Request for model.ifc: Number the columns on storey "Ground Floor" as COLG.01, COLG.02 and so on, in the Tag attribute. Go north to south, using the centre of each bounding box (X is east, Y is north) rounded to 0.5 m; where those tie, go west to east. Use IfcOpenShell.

First a look at what the model holds.

```python
import ifcopenshell
import ifcopenshell.util.element
import ifcopenshell.util.placement

model = ifcopenshell.open("model.ifc")
print(model.schema)
storey = next(s for s in model.by_type("IfcBuildingStorey") if s.Name == "Ground Floor")
columns = [e for e in ifcopenshell.util.element.get_decomposition(storey) if e.is_a("IfcColumn")]
for e in sorted(columns, key=lambda e: e.id()):
    origin = ifcopenshell.util.placement.get_local_placement(e.ObjectPlacement)[:3, 3]
    print(e.id(), e.Tag, e.Name, origin.round(2) + 0.0, sep=" | ")
```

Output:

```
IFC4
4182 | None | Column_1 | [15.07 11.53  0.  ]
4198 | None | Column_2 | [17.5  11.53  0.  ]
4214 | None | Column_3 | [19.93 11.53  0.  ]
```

```python
import ifcopenshell
import ifcopenshell.geom
import ifcopenshell.util.element
import ifcopenshell.util.shape

model = ifcopenshell.open("model.ifc")
settings = ifcopenshell.geom.settings()
settings.set("use-world-coords", True)


def centre(element):
    shape = ifcopenshell.geom.create_shape(settings, element)
    return ifcopenshell.util.shape.get_bbox_centroid(shape.geometry)


storey = next(s for s in model.by_type("IfcBuildingStorey") if s.Name == "Ground Floor")
columns = [e for e in ifcopenshell.util.element.get_decomposition(storey) if e.is_a("IfcColumn")]

# Insertion points can sit at a corner or the storey origin, so sort by the geometry (in metres).
centres = {e: centre(e) for e in columns}
columns.sort(key=lambda e: (-round(centres[e][1] / 0.5), centres[e][0]))

for i, e in enumerate(columns, start=1):
    number = f"COLG.{i:02d}"
    e.Tag = number
    print(e.id(), number)

model.write("model_updated.ifc")
```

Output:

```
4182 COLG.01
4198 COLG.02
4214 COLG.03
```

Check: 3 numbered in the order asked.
